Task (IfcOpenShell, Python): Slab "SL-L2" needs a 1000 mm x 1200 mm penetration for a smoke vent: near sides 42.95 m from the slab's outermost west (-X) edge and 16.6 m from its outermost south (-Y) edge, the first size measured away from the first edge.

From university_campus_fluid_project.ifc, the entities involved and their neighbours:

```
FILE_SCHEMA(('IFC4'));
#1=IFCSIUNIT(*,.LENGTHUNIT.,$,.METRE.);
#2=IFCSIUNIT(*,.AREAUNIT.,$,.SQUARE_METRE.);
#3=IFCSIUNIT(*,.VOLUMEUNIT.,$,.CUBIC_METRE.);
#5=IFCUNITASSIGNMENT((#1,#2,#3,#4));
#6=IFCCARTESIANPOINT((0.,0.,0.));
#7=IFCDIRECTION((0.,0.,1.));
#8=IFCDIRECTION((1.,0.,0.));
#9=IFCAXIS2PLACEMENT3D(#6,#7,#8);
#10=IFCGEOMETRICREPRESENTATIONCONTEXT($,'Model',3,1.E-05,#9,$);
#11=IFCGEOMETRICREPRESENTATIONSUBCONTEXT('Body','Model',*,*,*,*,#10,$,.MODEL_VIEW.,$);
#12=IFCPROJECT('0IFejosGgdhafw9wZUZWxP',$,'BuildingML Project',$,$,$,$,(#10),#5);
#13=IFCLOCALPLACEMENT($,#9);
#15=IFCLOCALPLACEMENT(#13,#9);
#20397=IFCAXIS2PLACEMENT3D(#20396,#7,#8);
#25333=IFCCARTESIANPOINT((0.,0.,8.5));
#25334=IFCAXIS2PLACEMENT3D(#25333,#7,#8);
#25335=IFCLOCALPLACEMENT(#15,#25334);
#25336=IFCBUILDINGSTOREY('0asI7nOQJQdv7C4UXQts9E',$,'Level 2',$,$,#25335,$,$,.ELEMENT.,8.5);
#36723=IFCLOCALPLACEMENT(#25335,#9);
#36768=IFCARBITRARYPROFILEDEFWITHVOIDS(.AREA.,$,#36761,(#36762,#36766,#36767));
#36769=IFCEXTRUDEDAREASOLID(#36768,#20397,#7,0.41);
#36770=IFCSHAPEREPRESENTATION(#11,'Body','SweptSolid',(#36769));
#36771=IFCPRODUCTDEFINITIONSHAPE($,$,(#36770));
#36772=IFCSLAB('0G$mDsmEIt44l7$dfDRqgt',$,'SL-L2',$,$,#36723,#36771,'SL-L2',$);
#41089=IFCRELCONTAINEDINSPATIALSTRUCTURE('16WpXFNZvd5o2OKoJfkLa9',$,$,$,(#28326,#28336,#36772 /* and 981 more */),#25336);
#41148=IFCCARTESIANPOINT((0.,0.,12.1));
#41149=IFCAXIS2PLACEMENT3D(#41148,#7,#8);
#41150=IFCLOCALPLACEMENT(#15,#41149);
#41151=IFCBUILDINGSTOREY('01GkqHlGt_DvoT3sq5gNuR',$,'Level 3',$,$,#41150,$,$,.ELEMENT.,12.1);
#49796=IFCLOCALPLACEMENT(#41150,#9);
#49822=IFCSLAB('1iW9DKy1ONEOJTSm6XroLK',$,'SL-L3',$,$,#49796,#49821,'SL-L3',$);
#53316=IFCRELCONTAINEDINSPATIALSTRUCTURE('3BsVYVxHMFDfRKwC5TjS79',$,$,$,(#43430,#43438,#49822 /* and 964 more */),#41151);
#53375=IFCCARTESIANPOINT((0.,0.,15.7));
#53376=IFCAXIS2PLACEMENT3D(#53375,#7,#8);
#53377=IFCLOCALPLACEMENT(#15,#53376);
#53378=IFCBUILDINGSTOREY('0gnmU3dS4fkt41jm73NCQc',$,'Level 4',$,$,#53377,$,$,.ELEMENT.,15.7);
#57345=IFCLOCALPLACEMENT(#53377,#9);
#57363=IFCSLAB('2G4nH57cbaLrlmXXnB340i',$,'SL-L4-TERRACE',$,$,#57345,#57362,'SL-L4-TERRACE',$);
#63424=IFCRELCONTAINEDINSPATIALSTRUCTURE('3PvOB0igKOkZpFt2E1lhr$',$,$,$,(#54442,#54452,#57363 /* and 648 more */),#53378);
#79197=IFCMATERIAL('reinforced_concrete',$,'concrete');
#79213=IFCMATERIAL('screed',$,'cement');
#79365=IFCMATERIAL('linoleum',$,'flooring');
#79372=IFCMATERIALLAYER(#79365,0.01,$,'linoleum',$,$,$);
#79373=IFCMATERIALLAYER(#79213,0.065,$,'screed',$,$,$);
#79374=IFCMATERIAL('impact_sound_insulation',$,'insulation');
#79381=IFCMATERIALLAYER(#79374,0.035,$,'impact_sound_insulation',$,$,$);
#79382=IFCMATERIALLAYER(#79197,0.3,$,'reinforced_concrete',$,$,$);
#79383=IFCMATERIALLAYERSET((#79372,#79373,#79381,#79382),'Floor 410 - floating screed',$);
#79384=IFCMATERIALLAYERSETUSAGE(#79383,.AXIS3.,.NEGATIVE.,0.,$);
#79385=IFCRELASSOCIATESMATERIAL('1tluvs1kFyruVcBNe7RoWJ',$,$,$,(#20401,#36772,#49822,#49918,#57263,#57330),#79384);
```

```python
import numpy as np
import ifcopenshell
import ifcopenshell.api.feature
import ifcopenshell.api.geometry
import ifcopenshell.api.root
import ifcopenshell.geom
import ifcopenshell.util.placement
import ifcopenshell.util.representation
import ifcopenshell.util.shape
import ifcopenshell.util.unit

model = ifcopenshell.open("university_campus_fluid_project.ifc")
unit_scale = ifcopenshell.util.unit.calculate_unit_scale(model)
settings = ifcopenshell.geom.settings()


def volume(element):
    """Net volume in cubic metres, openings subtracted."""
    shape = ifcopenshell.geom.create_shape(settings, element)
    return ifcopenshell.util.shape.get_volume(shape.geometry)


slab = model.by_guid("0G$mDsmEIt44l7$dfDRqgt")
before = volume(slab)

# Extent in the slab's own axes, in metres. The edges named are its -X and -Y sides.
slab_shape = ifcopenshell.geom.create_shape(settings, slab)
vertices = ifcopenshell.util.shape.get_vertices(slab_shape.geometry)
x_min, y_min, bottom = vertices.min(axis=0)
top = vertices[:, 2].max()

opening = ifcopenshell.api.root.create_entity(model, ifc_class="IfcOpeningElement", name="Smoke vent opening", predefined_type="OPENING")
context = ifcopenshell.util.representation.get_context(model, "Model", "Body", "MODEL_VIEW")
width, depth = 1, 1.2
outline = [(0.0, 0.0), (width, 0.0), (width, depth), (0.0, depth), (0.0, 0.0)]
# Overshoot both faces by 50 mm so the cut is clean.
shape = ifcopenshell.api.geometry.add_slab_representation(
    model, context=context, depth=top - bottom + 0.1, polyline=outline
)
ifcopenshell.api.geometry.assign_representation(model, product=opening, representation=shape)

matrix = ifcopenshell.util.placement.get_local_placement(slab.ObjectPlacement)
matrix[:, 3] = matrix @ np.append(np.array([x_min + 42.95, y_min + 16.6, bottom - 0.05]) / unit_scale, 1.0)
ifcopenshell.api.geometry.edit_object_placement(model, product=opening, matrix=matrix, is_si=False)
ifcopenshell.api.feature.add_feature(model, feature=opening, element=slab)

after = volume(slab)

print(f"slab volume {before:.3f} -> {after:.3f} m3")

model.write("university_campus_fluid_project_edited.ifc")
```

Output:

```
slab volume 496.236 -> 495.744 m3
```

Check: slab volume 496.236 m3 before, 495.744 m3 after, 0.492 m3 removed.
